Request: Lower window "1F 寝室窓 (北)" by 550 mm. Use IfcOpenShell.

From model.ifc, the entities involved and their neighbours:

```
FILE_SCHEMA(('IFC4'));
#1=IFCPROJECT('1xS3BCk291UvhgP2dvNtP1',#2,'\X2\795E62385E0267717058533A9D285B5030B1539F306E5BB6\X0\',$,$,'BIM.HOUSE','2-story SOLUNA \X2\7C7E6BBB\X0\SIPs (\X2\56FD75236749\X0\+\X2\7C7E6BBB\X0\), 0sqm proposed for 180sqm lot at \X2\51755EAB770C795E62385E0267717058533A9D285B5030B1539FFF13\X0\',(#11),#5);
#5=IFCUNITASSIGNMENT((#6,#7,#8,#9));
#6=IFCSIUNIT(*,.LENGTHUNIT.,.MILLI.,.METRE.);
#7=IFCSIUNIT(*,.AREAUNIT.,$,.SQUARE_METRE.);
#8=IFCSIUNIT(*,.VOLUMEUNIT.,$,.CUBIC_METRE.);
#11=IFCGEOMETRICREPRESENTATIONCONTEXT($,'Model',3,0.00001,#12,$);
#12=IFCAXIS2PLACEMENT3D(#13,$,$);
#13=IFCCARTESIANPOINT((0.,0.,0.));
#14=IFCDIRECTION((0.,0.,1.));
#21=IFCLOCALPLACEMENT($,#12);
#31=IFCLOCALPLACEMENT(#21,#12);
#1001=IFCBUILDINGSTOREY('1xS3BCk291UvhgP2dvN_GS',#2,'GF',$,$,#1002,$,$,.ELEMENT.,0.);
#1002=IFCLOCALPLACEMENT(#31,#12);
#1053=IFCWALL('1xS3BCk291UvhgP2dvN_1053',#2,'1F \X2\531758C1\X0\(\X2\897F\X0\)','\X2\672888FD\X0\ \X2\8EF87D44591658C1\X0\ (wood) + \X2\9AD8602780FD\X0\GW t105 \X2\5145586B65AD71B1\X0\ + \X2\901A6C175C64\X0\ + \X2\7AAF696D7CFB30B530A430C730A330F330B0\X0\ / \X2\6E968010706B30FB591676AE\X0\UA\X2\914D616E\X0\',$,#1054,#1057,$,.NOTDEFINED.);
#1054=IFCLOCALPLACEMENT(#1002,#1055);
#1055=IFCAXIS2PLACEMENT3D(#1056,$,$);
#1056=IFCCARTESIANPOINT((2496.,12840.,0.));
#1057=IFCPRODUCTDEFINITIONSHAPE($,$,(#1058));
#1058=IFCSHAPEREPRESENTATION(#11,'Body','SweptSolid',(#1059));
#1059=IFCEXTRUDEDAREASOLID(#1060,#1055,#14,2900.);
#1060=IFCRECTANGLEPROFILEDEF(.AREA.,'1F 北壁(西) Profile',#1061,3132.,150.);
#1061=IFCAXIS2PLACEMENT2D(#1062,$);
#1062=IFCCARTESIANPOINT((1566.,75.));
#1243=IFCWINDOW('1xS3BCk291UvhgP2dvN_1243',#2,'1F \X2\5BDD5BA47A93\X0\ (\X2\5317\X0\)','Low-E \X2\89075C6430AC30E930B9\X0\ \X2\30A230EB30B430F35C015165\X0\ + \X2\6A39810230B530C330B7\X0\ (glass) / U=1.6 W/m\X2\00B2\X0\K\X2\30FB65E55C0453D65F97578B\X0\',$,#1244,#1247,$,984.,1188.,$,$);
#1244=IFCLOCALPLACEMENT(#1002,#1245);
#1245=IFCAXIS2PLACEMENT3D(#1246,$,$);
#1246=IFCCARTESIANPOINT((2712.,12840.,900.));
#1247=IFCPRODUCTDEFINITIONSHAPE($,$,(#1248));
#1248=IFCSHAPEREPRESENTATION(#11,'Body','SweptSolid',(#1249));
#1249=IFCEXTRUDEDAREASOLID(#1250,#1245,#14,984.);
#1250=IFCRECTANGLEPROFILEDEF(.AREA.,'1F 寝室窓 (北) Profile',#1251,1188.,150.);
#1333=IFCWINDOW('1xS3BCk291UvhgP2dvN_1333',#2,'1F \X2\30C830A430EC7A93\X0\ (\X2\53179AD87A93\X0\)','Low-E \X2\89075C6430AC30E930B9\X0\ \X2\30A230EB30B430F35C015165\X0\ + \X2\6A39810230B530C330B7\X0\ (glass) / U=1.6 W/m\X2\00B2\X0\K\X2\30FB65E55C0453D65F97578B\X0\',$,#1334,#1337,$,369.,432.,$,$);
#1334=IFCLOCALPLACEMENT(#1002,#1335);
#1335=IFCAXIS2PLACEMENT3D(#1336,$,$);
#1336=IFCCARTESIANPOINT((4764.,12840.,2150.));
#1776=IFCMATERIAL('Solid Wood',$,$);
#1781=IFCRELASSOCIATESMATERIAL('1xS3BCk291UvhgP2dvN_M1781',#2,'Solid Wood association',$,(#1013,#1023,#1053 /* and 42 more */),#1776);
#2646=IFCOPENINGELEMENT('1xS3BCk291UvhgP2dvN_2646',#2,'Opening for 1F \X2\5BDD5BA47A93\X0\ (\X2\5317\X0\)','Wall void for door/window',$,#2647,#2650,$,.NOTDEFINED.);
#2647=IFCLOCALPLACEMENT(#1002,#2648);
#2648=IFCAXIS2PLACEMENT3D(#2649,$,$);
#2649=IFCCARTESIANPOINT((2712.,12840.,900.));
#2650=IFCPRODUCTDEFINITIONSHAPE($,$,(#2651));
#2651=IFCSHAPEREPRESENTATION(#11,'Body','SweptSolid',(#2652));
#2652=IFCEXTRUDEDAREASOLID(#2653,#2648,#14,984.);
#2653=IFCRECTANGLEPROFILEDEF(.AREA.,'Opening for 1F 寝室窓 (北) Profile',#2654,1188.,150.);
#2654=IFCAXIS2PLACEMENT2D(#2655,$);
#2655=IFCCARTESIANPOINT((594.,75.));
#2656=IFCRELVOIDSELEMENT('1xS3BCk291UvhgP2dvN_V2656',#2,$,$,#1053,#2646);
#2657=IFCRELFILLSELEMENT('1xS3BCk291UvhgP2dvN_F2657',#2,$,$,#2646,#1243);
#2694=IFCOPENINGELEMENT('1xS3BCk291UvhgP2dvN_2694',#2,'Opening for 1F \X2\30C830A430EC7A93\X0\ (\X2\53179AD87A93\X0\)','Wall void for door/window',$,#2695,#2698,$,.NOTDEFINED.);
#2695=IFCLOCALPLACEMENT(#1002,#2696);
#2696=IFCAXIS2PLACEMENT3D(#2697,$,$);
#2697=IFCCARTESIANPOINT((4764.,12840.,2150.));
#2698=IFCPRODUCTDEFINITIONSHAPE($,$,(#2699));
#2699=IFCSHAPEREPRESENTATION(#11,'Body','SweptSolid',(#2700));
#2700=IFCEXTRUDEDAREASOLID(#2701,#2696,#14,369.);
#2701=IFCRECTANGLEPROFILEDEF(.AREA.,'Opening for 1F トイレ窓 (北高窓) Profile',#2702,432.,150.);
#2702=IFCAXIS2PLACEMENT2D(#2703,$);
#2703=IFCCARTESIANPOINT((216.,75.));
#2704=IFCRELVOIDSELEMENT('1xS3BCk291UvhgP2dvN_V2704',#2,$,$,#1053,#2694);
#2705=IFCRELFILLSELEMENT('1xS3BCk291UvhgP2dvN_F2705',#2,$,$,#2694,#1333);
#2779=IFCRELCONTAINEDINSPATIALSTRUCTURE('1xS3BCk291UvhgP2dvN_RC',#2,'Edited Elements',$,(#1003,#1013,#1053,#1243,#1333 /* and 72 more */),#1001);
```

```python
import numpy as np
import ifcopenshell
import ifcopenshell.api.geometry
import ifcopenshell.util.placement
import ifcopenshell.util.unit

model = ifcopenshell.open("model.ifc")
unit_scale = ifcopenshell.util.unit.calculate_unit_scale(model)

window = model.by_guid("1xS3BCk291UvhgP2dvN_1243")
opening = window.FillsVoids[0].RelatingOpeningElement
dz = -0.55 / unit_scale

shift = np.array([0.0, 0.0, dz])
# The window is not placed relative to its opening, so move both.
for product in (opening, window):
    matrix = ifcopenshell.util.placement.get_local_placement(product.ObjectPlacement)
    matrix[:3, 3] += shift
    ifcopenshell.api.geometry.edit_object_placement(model, product=product, matrix=matrix, is_si=False)

print(f"moved by {dz * unit_scale:+.3f} m")

model.write("model_v2.ifc")
```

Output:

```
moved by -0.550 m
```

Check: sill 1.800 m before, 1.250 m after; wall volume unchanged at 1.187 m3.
